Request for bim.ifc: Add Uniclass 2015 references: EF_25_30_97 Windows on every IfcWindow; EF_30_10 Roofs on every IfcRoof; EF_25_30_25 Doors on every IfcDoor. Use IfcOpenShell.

First a look at what the model holds.

```python
import ifcopenshell

model = ifcopenshell.open("bim.ifc")
print(model.schema)
print("classifications:", [c.Name for c in model.by_type("IfcClassification")])
for ifc_class in ("IfcDoor", "IfcRoof", "IfcStair", "IfcWall", "IfcWindow"):
    print(ifc_class, len(model.by_type(ifc_class)))
```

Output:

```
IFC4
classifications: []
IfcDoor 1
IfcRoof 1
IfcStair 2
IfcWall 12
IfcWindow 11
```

```python
import ifcopenshell
import ifcopenshell.api.classification

model = ifcopenshell.open("bim.ifc")

system = ifcopenshell.api.classification.add_classification(model, classification="Uniclass 2015")

codes = {
    "IfcWindow": ("EF_25_30_97", "Windows"),
    "IfcRoof": ("EF_30_10", "Roofs"),
    "IfcDoor": ("EF_25_30_25", "Doors"),
}
for ifc_class, (code, name) in codes.items():
    products = model.by_type(ifc_class)
    ifcopenshell.api.classification.add_reference(
        model, products=products, classification=system, identification=code, name=name
    )
    print(code, len(products))

model.write("bim_edited.ifc")
```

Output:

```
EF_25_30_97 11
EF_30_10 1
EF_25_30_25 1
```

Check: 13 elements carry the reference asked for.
